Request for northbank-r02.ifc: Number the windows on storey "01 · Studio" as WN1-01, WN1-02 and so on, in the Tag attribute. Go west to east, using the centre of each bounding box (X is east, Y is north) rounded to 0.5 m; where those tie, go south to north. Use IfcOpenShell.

First a look at what the model holds.

```python
import ifcopenshell
import ifcopenshell.util.element
import ifcopenshell.util.placement

model = ifcopenshell.open("northbank-r02.ifc")
print(model.schema)
storey = next(s for s in model.by_type("IfcBuildingStorey") if s.Name == "01 · Studio")
windows = [e for e in ifcopenshell.util.element.get_decomposition(storey) if e.is_a("IfcWindow")]
for e in sorted(windows, key=lambda e: e.id()):
    origin = ifcopenshell.util.placement.get_local_placement(e.ObjectPlacement)[:3, 3]
    print(e.id(), e.Tag, e.Name, origin.round(2) + 0.0, sep=" | ")
```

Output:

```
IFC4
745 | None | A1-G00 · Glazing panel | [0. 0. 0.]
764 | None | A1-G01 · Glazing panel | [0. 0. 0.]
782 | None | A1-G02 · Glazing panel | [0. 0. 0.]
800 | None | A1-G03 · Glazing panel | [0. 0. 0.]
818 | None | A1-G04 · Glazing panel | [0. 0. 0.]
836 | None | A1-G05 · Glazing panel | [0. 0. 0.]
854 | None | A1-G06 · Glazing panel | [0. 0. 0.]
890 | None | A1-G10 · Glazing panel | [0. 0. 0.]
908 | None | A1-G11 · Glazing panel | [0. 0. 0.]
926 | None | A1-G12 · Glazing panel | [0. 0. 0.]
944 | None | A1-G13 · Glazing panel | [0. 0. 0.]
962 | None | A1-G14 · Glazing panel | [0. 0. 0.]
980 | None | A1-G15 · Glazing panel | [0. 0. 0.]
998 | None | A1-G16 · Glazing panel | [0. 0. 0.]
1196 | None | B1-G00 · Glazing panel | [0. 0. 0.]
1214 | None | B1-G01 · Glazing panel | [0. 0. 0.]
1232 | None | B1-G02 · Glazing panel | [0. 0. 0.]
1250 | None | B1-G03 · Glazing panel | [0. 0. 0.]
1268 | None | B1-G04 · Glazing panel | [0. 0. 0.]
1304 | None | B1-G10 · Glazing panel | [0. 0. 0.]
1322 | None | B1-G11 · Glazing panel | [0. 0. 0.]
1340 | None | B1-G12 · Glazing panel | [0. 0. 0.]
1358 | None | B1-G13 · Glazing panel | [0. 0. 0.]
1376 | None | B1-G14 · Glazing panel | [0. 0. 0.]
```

```python
import ifcopenshell
import ifcopenshell.geom
import ifcopenshell.util.element
import ifcopenshell.util.shape

model = ifcopenshell.open("northbank-r02.ifc")
settings = ifcopenshell.geom.settings()
settings.set("use-world-coords", True)


def centre(element):
    shape = ifcopenshell.geom.create_shape(settings, element)
    return ifcopenshell.util.shape.get_bbox_centroid(shape.geometry)


storey = next(s for s in model.by_type("IfcBuildingStorey") if s.Name == "01 · Studio")
windows = [e for e in ifcopenshell.util.element.get_decomposition(storey) if e.is_a("IfcWindow")]

# Insertion points can sit at a corner or the storey origin, so sort by the geometry (in metres).
centres = {e: centre(e) for e in windows}
windows.sort(key=lambda e: (round(centres[e][0] / 0.5), centres[e][1]))

for i, e in enumerate(windows, start=1):
    number = f"WN1-{i:02d}"
    e.Tag = number
    print(e.id(), number)

model.write("northbank-r02_edited.ifc")
```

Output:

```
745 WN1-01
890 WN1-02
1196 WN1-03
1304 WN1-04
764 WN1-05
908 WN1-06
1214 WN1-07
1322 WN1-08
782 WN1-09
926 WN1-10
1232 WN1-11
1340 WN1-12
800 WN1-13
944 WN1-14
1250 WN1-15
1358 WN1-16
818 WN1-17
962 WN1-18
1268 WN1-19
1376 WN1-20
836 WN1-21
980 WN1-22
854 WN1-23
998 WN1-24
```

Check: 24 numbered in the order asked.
